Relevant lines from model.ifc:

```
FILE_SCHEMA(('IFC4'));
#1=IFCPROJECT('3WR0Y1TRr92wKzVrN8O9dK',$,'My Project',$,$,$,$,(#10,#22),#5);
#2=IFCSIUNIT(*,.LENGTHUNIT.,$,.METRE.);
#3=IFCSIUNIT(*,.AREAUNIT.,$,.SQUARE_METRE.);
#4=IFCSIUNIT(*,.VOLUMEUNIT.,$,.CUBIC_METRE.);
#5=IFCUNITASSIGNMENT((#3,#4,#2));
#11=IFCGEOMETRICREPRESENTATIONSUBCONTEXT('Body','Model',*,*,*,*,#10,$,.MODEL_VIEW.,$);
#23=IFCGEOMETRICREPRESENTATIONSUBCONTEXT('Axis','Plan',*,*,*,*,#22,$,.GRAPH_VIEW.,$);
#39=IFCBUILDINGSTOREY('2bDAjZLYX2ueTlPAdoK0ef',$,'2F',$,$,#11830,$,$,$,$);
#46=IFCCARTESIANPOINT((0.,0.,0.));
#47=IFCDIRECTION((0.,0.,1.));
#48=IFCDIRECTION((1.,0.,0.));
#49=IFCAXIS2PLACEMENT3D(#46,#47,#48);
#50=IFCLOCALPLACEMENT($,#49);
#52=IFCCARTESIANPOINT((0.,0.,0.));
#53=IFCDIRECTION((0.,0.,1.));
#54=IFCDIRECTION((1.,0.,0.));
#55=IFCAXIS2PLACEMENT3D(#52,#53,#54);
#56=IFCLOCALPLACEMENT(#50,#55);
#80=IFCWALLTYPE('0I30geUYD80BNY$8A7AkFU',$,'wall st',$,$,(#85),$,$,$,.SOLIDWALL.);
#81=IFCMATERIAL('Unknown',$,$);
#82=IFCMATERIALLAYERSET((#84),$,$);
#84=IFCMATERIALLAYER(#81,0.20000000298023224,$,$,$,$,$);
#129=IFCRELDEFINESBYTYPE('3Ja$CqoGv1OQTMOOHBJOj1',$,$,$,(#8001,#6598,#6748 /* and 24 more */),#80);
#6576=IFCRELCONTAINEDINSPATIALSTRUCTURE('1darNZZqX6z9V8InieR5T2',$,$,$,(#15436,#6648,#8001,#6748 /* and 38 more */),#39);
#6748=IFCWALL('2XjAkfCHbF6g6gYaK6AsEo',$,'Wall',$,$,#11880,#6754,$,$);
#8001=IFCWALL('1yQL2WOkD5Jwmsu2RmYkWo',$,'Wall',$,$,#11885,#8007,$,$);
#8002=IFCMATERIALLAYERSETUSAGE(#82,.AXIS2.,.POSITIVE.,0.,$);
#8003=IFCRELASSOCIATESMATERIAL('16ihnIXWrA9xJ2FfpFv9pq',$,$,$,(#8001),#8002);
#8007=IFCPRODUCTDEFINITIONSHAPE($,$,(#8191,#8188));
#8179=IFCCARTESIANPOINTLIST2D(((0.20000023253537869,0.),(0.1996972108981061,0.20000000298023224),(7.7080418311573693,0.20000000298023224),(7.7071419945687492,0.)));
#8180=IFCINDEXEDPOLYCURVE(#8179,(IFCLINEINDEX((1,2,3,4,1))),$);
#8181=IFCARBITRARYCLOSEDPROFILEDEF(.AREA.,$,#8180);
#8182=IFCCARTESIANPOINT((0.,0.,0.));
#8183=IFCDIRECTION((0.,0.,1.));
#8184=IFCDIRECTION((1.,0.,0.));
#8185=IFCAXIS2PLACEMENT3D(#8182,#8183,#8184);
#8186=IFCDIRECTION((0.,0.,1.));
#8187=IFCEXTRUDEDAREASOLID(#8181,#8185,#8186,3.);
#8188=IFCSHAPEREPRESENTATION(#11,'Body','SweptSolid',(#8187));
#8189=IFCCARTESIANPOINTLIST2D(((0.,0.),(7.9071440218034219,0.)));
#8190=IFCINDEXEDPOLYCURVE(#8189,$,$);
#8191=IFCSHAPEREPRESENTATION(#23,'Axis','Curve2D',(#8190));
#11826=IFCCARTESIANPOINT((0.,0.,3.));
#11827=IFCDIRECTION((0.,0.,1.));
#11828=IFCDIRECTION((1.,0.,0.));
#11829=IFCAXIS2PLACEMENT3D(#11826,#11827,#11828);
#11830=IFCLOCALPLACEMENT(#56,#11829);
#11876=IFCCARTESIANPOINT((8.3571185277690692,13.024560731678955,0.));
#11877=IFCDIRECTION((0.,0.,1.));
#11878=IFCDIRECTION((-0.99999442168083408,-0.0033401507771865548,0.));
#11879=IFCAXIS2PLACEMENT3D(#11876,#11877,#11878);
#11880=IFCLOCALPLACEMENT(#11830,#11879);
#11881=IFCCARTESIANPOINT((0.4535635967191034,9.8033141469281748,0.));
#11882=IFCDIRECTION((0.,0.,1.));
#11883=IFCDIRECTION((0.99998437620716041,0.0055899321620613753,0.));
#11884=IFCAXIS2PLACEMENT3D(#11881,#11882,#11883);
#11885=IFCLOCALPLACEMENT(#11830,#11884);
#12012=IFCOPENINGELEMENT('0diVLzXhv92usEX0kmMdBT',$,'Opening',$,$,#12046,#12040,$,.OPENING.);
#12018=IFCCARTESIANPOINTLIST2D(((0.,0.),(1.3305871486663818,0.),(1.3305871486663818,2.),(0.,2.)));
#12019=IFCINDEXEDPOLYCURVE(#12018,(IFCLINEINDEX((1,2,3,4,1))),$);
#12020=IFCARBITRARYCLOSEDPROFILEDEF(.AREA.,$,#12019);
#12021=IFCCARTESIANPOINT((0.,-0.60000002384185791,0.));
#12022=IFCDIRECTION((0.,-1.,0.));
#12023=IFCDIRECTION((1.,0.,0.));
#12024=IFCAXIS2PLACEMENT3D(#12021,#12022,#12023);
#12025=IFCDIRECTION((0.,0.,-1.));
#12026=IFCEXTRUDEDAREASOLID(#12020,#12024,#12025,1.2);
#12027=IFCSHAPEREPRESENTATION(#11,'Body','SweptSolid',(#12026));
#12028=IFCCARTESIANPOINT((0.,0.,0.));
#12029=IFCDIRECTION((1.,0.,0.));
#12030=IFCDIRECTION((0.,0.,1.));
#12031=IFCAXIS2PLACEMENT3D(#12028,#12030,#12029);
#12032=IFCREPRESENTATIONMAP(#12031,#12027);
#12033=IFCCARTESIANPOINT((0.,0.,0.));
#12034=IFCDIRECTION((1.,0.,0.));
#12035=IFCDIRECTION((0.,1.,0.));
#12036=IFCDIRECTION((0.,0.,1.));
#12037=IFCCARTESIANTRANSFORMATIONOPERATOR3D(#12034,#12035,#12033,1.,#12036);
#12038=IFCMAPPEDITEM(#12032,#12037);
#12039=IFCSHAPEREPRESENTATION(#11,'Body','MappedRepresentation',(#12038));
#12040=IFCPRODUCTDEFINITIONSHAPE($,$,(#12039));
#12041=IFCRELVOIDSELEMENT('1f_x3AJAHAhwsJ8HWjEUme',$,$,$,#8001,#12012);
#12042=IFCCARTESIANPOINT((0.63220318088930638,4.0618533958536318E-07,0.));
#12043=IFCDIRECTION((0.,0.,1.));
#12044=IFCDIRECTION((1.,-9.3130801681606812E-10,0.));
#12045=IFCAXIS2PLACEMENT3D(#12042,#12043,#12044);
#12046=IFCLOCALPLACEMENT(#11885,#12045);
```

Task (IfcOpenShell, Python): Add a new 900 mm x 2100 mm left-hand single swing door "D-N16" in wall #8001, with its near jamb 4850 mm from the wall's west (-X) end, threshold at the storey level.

```python
import numpy as np
import ifcopenshell
import ifcopenshell.api.feature
import ifcopenshell.api.geometry
import ifcopenshell.api.root
import ifcopenshell.api.spatial
import ifcopenshell.geom
import ifcopenshell.util.element
import ifcopenshell.util.placement
import ifcopenshell.util.representation
import ifcopenshell.util.shape
import ifcopenshell.util.unit

model = ifcopenshell.open("model.ifc")
unit_scale = ifcopenshell.util.unit.calculate_unit_scale(model)
settings = ifcopenshell.geom.settings()


def volume(element):
    """Net volume in cubic metres, openings subtracted."""
    shape = ifcopenshell.geom.create_shape(settings, element)
    return ifcopenshell.util.shape.get_volume(shape.geometry)


wall = model.by_guid("1yQL2WOkD5Jwmsu2RmYkWo")
storey = ifcopenshell.util.element.get_container(wall, ifc_class="IfcBuildingStorey")
context = ifcopenshell.util.representation.get_context(model, "Model", "Body", "MODEL_VIEW")
before = volume(wall)

width, height, from_end, sill = 0.9, 2.1, 4.85, 0.0  # metres

# The wall runs along its own X axis, and the end named is its -X end.
wall_shape = ifcopenshell.geom.create_shape(settings, wall)
x, y, z = ifcopenshell.util.shape.get_vertices(wall_shape.geometry).T
start = x.min() + from_end
face, thickness = float(y.min()), float(y.max() - y.min())
wall_matrix = ifcopenshell.util.placement.get_local_placement(wall.ObjectPlacement)
level = ifcopenshell.util.placement.get_local_placement(storey.ObjectPlacement)[2, 3]


def in_wall(x, y):
    """Placement at x, y metres in the wall's axes, at sill height."""
    matrix = wall_matrix.copy()
    matrix[:, 3] = wall_matrix @ np.array([x / unit_scale, y / unit_scale, 0.0, 1.0])
    matrix[2, 3] = level + sill / unit_scale
    return matrix


# Opening: a box that overshoots both wall faces by 50 mm.
opening = ifcopenshell.api.root.create_entity(model, ifc_class="IfcOpeningElement", predefined_type="OPENING")
box = ifcopenshell.api.geometry.add_wall_representation(
    model, context=context, length=width, height=height, thickness=thickness + 0.1
)
ifcopenshell.api.geometry.assign_representation(model, product=opening, representation=box)
ifcopenshell.api.geometry.edit_object_placement(model, product=opening, matrix=in_wall(start, face - 0.05), is_si=False)
ifcopenshell.api.feature.add_feature(model, feature=opening, element=wall)

door = ifcopenshell.api.root.create_entity(model, ifc_class="IfcDoor", name="D-N16", predefined_type="DOOR")
door.OverallWidth, door.OverallHeight = width / unit_scale, height / unit_scale
door.OperationType = "SINGLE_SWING_LEFT"
body = ifcopenshell.api.geometry.add_door_representation(
    model,
    context=context,
    overall_width=door.OverallWidth,
    overall_height=door.OverallHeight,
    operation_type="SINGLE_SWING_LEFT",
    lining_properties={"LiningDepth": thickness / unit_scale, "ThresholdDepth": thickness / unit_scale},
)
ifcopenshell.api.geometry.assign_representation(model, product=door, representation=body)
ifcopenshell.api.spatial.assign_container(model, products=[door], relating_structure=storey)
ifcopenshell.api.feature.add_filling(model, opening=opening, element=door)

# The lining spans the wall, so the door starts at the wall face.
ifcopenshell.api.geometry.edit_object_placement(model, product=door, matrix=in_wall(start, face), is_si=False)

after = volume(wall)

print(f"wall volume {before:.3f} -> {after:.3f} m3")

model.write("model_rev.ifc")
```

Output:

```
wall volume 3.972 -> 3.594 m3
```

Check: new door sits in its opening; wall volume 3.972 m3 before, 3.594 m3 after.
